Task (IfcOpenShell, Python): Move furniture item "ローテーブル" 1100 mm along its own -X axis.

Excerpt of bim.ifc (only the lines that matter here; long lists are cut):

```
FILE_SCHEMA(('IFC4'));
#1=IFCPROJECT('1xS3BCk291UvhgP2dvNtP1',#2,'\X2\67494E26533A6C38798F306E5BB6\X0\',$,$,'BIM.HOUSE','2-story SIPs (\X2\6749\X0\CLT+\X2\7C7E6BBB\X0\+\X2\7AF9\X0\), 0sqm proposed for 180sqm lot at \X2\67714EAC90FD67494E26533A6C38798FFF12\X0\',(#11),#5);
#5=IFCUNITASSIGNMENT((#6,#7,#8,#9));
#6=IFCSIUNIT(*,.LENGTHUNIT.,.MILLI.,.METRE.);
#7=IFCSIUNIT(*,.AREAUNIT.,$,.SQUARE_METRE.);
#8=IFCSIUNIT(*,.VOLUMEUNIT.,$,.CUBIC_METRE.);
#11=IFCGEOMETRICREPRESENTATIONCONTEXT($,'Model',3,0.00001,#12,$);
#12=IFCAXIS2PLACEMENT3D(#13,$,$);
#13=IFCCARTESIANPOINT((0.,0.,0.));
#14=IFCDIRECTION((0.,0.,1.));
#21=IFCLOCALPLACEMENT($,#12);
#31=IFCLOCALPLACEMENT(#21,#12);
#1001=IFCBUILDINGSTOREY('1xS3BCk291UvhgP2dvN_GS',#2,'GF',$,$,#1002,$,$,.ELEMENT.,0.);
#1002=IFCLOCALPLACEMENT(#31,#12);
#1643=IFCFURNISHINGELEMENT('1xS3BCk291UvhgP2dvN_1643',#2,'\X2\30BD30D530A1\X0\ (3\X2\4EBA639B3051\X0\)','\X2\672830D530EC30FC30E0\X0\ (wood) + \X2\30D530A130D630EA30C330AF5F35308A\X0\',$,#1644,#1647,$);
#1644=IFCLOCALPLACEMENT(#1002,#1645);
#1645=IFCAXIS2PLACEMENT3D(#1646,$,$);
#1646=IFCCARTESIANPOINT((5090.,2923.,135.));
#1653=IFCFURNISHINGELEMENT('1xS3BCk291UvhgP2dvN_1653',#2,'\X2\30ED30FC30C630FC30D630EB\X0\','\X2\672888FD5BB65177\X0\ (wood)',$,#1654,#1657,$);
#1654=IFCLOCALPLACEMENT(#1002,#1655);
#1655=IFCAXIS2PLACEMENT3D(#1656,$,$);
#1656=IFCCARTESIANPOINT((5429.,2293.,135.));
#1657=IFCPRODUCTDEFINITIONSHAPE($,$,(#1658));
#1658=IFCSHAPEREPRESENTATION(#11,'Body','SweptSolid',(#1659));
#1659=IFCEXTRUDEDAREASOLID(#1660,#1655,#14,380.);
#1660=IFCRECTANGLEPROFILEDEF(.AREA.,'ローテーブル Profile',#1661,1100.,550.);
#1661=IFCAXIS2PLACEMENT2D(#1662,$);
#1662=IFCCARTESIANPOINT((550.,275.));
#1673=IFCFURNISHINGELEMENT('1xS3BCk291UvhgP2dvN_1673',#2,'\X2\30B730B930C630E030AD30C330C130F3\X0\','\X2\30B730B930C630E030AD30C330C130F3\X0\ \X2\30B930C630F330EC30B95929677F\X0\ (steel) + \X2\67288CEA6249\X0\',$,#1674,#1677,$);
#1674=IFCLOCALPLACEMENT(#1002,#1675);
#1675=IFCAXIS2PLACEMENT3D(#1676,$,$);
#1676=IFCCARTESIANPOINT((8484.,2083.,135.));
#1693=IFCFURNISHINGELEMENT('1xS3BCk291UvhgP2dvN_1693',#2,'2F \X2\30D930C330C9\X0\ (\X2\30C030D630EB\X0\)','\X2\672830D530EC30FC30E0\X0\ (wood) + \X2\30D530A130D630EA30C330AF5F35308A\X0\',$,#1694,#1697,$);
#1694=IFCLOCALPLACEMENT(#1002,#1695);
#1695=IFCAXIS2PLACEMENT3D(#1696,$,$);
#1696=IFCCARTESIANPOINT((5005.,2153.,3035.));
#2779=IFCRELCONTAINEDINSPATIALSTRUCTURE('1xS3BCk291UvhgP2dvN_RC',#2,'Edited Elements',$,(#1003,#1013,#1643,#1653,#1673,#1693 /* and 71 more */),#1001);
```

```python
import ifcopenshell
import ifcopenshell.api.geometry
import ifcopenshell.util.placement
import ifcopenshell.util.unit

model = ifcopenshell.open("bim.ifc")
unit_scale = ifcopenshell.util.unit.calculate_unit_scale(model)

item = model.by_guid("1xS3BCk291UvhgP2dvN_1653")
matrix = ifcopenshell.util.placement.get_local_placement(item.ObjectPlacement)
matrix[:3, 3] -= matrix[:3, 0] * 1.1 / unit_scale
ifcopenshell.api.geometry.edit_object_placement(model, product=item, matrix=matrix, is_si=False)

print(ifcopenshell.util.placement.get_local_placement(item.ObjectPlacement).round(3) + 0.0)

model.write("bim-out.ifc")
```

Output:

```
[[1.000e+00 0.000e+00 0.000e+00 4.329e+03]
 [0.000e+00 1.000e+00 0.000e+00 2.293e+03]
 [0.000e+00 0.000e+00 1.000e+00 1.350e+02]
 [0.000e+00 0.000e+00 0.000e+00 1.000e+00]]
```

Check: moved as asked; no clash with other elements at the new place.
